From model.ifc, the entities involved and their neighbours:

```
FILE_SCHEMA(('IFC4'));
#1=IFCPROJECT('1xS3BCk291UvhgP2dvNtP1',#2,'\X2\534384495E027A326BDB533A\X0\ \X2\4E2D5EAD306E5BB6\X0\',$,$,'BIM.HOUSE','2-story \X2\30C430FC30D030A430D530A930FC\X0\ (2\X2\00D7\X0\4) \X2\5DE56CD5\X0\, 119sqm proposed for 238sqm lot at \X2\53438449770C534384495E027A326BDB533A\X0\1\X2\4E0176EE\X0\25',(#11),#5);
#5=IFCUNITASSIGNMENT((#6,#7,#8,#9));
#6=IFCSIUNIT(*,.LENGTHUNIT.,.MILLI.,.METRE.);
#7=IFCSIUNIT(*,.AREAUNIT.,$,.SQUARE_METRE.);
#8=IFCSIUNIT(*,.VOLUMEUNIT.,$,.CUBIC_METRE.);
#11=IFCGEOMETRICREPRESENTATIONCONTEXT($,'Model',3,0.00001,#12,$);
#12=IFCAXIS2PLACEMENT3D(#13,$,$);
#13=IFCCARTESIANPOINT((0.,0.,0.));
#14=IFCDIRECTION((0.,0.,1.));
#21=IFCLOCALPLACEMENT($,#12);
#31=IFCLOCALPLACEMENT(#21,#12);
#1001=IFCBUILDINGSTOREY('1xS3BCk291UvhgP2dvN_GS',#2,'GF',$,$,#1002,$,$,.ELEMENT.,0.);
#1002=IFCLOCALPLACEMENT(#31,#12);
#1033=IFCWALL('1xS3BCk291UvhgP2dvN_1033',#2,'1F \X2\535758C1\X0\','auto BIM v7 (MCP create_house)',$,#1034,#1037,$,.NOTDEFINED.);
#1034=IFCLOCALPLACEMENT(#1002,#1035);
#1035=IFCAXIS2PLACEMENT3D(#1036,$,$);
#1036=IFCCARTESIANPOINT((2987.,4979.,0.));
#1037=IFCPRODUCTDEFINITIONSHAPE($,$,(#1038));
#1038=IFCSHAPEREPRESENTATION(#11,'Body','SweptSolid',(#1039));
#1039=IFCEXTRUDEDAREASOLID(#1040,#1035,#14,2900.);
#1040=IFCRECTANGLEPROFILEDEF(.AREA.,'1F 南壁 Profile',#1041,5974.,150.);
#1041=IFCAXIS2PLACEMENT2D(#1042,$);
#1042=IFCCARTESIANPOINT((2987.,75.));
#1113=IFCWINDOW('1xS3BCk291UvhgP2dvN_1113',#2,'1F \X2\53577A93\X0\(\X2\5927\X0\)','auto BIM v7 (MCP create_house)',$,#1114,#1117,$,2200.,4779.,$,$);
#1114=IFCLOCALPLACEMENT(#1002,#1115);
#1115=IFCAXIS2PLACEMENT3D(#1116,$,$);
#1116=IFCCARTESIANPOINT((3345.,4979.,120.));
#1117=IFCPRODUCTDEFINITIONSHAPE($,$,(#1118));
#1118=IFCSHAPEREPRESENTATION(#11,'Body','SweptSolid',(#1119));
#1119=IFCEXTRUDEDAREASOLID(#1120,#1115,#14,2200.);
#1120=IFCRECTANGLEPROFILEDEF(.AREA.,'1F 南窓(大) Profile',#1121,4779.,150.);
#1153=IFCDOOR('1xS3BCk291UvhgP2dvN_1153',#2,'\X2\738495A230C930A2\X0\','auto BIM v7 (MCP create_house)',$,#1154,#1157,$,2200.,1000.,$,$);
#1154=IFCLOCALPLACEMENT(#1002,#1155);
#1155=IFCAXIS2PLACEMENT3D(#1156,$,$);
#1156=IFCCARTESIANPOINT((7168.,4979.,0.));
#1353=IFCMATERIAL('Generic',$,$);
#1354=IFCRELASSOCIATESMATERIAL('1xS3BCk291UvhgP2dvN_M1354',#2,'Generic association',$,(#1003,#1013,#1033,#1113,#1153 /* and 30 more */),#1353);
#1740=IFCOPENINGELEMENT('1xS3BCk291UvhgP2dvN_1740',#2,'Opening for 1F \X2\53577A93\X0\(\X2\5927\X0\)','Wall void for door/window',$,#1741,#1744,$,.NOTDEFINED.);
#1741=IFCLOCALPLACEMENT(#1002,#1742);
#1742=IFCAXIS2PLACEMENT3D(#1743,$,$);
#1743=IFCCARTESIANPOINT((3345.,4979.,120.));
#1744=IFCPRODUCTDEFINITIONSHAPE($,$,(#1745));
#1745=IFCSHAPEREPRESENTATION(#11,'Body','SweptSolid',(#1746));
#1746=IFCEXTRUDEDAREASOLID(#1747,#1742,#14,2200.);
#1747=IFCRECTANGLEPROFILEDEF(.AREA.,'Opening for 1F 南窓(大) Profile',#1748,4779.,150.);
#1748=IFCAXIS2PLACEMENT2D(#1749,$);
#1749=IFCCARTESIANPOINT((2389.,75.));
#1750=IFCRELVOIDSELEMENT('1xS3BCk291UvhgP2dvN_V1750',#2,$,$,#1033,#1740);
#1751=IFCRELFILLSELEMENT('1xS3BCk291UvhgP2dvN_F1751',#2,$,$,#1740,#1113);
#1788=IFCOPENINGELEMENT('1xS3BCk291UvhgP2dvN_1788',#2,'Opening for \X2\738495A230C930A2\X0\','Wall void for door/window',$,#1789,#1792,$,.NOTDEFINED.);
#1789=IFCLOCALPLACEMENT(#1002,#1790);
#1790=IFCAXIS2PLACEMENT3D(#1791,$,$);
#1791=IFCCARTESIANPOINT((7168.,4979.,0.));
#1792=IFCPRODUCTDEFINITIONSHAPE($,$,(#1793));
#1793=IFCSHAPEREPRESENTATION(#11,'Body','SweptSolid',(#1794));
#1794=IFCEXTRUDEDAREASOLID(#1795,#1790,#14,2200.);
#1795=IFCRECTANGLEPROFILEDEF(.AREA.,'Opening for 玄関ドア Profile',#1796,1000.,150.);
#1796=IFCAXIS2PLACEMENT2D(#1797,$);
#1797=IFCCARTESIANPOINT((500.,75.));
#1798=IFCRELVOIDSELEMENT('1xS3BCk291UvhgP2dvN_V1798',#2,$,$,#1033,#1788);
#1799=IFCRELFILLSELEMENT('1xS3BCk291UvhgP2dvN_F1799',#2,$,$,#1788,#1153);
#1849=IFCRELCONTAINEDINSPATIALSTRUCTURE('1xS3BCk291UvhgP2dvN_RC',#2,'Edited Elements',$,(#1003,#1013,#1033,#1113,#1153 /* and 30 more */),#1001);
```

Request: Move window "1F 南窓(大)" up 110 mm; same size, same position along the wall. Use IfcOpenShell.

```python
import numpy as np
import ifcopenshell
import ifcopenshell.api.geometry
import ifcopenshell.util.placement
import ifcopenshell.util.unit

model = ifcopenshell.open("model.ifc")
unit_scale = ifcopenshell.util.unit.calculate_unit_scale(model)

window = model.by_id(1113)
opening = window.FillsVoids[0].RelatingOpeningElement
dz = 0.11 / unit_scale

shift = np.array([0.0, 0.0, dz])
# The window is not placed relative to its opening, so move both.
for product in (opening, window):
    matrix = ifcopenshell.util.placement.get_local_placement(product.ObjectPlacement)
    matrix[:3, 3] += shift
    ifcopenshell.api.geometry.edit_object_placement(model, product=product, matrix=matrix, is_si=False)

print(f"moved by {dz * unit_scale:+.3f} m")

model.write("model_edited.ifc")
```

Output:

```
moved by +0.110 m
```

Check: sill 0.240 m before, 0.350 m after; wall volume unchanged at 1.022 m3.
